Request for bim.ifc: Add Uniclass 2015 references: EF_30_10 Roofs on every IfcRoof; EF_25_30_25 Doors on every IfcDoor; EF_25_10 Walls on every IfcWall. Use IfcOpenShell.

First a look at what the model holds.

```python
import ifcopenshell

model = ifcopenshell.open("bim.ifc")
print(model.schema)
print("classifications:", [c.Name for c in model.by_type("IfcClassification")])
for ifc_class in ("IfcDoor", "IfcRoof", "IfcStair", "IfcWall", "IfcWindow"):
    print(ifc_class, len(model.by_type(ifc_class)))
```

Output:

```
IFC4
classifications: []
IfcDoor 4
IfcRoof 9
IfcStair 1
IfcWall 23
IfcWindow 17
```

```python
import ifcopenshell
import ifcopenshell.api.classification

model = ifcopenshell.open("bim.ifc")

system = ifcopenshell.api.classification.add_classification(model, classification="Uniclass 2015")

codes = {
    "IfcRoof": ("EF_30_10", "Roofs"),
    "IfcDoor": ("EF_25_30_25", "Doors"),
    "IfcWall": ("EF_25_10", "Walls"),
}
for ifc_class, (code, name) in codes.items():
    products = model.by_type(ifc_class)
    ifcopenshell.api.classification.add_reference(
        model, products=products, classification=system, identification=code, name=name
    )
    print(code, len(products))

model.write("bim_v2.ifc")
```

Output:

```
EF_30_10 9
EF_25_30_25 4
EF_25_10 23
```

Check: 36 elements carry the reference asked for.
